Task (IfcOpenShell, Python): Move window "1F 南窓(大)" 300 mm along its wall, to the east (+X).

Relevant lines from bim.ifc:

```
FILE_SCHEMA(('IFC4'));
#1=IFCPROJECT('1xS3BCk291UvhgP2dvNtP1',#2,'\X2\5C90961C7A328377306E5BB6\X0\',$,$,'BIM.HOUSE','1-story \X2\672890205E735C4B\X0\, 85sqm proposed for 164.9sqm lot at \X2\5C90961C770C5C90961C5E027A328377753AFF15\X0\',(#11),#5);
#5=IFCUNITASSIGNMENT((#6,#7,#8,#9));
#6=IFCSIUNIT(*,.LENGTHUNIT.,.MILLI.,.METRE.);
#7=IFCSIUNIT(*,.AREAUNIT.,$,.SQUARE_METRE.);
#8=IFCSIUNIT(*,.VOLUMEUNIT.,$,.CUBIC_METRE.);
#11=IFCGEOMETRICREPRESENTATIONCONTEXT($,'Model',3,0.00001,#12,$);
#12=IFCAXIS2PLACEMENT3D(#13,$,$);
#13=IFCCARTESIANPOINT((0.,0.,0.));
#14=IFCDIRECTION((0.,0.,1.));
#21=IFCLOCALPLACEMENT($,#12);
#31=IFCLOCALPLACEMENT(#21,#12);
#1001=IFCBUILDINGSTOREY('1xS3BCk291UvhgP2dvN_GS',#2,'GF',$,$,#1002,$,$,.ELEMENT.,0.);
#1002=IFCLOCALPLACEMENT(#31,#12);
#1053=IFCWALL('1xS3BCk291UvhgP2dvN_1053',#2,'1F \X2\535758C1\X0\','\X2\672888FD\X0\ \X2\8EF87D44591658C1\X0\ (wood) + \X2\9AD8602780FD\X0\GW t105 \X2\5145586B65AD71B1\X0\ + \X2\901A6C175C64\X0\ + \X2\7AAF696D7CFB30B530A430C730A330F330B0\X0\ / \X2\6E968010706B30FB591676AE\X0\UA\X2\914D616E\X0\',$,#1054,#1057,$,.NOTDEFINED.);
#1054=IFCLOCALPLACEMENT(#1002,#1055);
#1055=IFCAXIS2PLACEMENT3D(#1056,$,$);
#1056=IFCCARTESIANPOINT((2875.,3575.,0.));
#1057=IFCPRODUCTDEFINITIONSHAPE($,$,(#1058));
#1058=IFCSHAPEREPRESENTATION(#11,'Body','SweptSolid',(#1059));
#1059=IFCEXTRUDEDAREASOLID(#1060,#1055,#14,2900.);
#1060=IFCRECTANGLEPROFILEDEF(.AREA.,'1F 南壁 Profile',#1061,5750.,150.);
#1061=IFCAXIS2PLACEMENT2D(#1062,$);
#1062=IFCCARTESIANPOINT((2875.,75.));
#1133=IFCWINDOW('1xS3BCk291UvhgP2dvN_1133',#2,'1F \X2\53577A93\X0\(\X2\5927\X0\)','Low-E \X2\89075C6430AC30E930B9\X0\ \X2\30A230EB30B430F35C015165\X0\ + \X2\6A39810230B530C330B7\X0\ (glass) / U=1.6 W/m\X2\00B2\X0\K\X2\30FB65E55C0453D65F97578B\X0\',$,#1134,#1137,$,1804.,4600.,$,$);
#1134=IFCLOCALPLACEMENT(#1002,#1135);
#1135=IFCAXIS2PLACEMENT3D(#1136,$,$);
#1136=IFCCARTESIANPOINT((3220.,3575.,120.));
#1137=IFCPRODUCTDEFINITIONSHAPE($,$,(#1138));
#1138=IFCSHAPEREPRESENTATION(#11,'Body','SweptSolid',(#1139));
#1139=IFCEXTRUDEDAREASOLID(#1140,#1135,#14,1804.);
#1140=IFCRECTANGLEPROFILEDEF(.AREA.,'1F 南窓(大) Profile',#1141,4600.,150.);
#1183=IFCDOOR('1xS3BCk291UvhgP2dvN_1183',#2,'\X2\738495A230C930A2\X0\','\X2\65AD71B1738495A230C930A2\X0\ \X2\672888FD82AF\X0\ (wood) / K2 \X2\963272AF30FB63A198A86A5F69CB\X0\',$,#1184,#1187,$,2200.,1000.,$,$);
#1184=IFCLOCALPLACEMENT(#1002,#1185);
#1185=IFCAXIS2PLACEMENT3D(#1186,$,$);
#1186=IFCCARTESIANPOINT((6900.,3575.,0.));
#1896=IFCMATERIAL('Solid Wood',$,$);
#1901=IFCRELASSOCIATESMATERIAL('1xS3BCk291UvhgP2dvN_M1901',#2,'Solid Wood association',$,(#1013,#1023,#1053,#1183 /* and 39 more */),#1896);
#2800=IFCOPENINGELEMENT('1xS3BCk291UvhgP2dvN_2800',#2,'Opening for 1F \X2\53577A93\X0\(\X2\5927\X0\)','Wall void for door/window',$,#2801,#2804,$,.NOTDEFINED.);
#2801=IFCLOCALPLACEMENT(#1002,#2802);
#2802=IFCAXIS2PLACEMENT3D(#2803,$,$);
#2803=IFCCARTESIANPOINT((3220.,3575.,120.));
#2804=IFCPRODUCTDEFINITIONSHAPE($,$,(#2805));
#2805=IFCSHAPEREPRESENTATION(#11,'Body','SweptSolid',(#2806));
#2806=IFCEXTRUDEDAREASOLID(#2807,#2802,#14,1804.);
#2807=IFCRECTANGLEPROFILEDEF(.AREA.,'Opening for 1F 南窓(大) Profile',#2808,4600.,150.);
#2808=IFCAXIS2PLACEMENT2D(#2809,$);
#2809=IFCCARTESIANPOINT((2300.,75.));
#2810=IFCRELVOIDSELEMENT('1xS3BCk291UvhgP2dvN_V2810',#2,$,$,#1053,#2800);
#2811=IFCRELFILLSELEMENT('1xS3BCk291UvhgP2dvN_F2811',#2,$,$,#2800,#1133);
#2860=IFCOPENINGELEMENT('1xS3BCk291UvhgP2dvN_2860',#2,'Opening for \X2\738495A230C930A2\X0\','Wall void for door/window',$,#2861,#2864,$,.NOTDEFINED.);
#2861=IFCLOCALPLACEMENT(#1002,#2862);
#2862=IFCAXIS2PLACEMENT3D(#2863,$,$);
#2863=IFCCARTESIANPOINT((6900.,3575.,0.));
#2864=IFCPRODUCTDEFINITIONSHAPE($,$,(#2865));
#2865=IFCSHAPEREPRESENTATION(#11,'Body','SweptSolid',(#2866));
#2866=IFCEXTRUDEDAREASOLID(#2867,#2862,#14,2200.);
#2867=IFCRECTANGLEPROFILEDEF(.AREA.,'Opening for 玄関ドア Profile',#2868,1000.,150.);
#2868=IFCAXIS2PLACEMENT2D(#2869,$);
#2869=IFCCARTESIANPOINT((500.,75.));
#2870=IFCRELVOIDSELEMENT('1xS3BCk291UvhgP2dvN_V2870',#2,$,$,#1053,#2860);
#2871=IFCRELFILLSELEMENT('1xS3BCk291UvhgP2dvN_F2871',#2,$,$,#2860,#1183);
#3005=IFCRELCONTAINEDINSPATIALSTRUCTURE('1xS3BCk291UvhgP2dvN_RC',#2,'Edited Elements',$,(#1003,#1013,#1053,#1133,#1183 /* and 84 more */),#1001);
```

```python
import ifcopenshell
import ifcopenshell.api.geometry
import ifcopenshell.util.placement
import ifcopenshell.util.unit

model = ifcopenshell.open("bim.ifc")
unit_scale = ifcopenshell.util.unit.calculate_unit_scale(model)

window = model.by_id(1133)
opening = window.FillsVoids[0].RelatingOpeningElement
wall = opening.VoidsElements[0].RelatingBuildingElement

wall_matrix = ifcopenshell.util.placement.get_local_placement(wall.ObjectPlacement)
shift = wall_matrix[:3, 0] * 0.3 / unit_scale
before = ifcopenshell.util.placement.get_local_placement(window.ObjectPlacement)[:3, 3].copy()

# The window is not placed relative to its opening, so move both.
for product in (opening, window):
    matrix = ifcopenshell.util.placement.get_local_placement(product.ObjectPlacement)
    matrix[:3, 3] += shift
    ifcopenshell.api.geometry.edit_object_placement(model, product=product, matrix=matrix, is_si=False)

after = ifcopenshell.util.placement.get_local_placement(window.ObjectPlacement)[:3, 3]
print("window moved by", (after - before).round(3) + 0.0)

model.write("bim_rev.ifc")
```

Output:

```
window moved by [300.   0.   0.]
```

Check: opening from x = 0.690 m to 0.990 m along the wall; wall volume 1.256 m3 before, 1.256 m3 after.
